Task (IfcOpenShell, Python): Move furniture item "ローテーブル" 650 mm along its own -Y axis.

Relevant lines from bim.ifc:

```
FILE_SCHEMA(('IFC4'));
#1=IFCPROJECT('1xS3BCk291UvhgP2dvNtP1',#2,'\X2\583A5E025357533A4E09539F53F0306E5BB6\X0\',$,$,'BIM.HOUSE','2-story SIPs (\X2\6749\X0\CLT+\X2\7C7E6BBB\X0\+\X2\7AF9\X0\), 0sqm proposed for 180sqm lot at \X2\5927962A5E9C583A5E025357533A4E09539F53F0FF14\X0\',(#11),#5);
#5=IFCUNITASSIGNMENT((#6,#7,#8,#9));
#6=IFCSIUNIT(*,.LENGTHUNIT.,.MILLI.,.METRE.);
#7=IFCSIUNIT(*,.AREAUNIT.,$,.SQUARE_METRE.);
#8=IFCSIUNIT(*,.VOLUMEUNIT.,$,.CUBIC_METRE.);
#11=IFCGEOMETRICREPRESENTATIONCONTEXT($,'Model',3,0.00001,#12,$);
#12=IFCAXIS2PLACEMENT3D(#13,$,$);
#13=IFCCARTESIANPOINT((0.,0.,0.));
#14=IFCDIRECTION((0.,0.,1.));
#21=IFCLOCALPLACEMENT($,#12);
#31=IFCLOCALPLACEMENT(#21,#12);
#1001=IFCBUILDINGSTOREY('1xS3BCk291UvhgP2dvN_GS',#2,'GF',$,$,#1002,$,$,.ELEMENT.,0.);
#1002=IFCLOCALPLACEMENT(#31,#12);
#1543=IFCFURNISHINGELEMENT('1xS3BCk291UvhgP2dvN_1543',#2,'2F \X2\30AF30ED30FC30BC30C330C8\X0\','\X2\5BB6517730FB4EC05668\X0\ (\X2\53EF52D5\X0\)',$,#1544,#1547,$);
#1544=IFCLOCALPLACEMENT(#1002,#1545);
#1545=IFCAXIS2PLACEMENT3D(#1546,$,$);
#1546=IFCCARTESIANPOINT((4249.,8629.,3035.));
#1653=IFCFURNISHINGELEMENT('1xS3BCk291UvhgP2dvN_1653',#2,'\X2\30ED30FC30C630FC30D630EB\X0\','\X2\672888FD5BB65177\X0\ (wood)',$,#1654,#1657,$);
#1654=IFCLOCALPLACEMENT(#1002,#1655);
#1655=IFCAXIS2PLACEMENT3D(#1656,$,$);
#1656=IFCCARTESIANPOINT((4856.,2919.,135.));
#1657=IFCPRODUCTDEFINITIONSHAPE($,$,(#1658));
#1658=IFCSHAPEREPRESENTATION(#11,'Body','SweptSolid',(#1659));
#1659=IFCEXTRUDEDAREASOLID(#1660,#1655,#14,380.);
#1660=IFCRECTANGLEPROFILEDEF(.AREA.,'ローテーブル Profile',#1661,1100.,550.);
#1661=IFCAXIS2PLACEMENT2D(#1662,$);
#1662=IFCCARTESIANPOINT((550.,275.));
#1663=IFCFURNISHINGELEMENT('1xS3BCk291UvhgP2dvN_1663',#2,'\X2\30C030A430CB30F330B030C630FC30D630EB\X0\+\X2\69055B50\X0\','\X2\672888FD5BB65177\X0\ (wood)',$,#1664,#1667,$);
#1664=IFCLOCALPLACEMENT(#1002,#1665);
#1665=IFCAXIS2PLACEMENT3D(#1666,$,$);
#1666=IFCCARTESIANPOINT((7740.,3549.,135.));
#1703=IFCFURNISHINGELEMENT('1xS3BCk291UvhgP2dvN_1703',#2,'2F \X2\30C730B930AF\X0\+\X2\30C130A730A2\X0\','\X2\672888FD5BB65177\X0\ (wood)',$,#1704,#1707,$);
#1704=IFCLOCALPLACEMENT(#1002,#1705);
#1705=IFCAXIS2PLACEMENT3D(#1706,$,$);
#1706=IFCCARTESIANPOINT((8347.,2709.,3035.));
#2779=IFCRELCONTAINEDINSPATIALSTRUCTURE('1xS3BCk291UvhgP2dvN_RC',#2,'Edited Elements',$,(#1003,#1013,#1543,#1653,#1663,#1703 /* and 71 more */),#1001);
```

```python
import ifcopenshell
import ifcopenshell.api.geometry
import ifcopenshell.util.placement
import ifcopenshell.util.unit

model = ifcopenshell.open("bim.ifc")
unit_scale = ifcopenshell.util.unit.calculate_unit_scale(model)

item = model.by_guid("1xS3BCk291UvhgP2dvN_1653")
matrix = ifcopenshell.util.placement.get_local_placement(item.ObjectPlacement)
matrix[:3, 3] -= matrix[:3, 1] * 0.65 / unit_scale
ifcopenshell.api.geometry.edit_object_placement(model, product=item, matrix=matrix, is_si=False)

print(ifcopenshell.util.placement.get_local_placement(item.ObjectPlacement).round(3) + 0.0)

model.write("bim_edited.ifc")
```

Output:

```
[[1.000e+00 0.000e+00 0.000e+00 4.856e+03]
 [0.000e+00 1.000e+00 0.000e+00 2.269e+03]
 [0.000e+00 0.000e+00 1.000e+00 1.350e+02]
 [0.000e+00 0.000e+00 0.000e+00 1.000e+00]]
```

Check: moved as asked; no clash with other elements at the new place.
